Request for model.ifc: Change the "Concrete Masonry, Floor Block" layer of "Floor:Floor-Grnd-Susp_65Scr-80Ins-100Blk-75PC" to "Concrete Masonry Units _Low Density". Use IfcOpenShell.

First a look at what the model holds.

```python
import ifcopenshell
import ifcopenshell.util.element

model = ifcopenshell.open("model.ifc")
print(model.schema)
for layer_set in model.by_type("IfcMaterialLayerSet"):
    if layer_set.LayerSetName == "Floor:Floor-Grnd-Susp_65Scr-80Ins-100Blk-75PC":
        for layer in layer_set.MaterialLayers:
            print(layer.id(), layer.Material and layer.Material.Name, layer.LayerThickness, sep=" | ")
        print(len(ifcopenshell.util.element.get_elements_by_material(model, layer_set)), "elements and types use it")
print(sorted(m.Name for m in model.by_type("IfcMaterial") if m.Name)[:60])
```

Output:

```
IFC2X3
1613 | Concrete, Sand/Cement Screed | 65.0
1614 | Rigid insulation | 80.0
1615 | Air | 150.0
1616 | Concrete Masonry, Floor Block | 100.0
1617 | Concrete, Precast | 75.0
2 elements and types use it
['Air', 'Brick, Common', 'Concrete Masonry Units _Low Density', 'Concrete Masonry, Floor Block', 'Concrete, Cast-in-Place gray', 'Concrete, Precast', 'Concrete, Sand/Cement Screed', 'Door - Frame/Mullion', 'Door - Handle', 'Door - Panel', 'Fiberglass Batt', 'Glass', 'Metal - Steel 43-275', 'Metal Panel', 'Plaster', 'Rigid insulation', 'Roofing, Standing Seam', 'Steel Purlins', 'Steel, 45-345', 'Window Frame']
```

```python
import ifcopenshell
import ifcopenshell.api.material

model = ifcopenshell.open("model.ifc")

layer_set = next(s for s in model.by_type("IfcMaterialLayerSet") if s.LayerSetName == "Floor:Floor-Grnd-Susp_65Scr-80Ins-100Blk-75PC")
layer = next(l for l in layer_set.MaterialLayers if l.Material and l.Material.Name == "Concrete Masonry, Floor Block")
material = next(m for m in model.by_type("IfcMaterial") if m.Name == "Concrete Masonry Units _Low Density")

# Point this one layer at the other material; renaming the old one would change it everywhere.
ifcopenshell.api.material.edit_layer(model, layer=layer, attributes={}, material=material)

print([l.Material.Name if l.Material else None for l in layer_set.MaterialLayers])

model.write("model_rev.ifc")
```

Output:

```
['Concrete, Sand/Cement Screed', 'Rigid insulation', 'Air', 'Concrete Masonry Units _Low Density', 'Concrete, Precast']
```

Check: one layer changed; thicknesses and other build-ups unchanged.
